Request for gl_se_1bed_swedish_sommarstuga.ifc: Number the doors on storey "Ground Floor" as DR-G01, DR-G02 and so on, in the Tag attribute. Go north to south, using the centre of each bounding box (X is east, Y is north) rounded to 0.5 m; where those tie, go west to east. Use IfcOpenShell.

First a look at what the model holds.

```python
import ifcopenshell
import ifcopenshell.util.element
import ifcopenshell.util.placement

model = ifcopenshell.open("gl_se_1bed_swedish_sommarstuga.ifc")
print(model.schema)
storey = next(s for s in model.by_type("IfcBuildingStorey") if s.Name == "Ground Floor")
doors = [e for e in ifcopenshell.util.element.get_decomposition(storey) if e.is_a("IfcDoor")]
for e in sorted(doors, key=lambda e: e.id()):
    origin = ifcopenshell.util.placement.get_local_placement(e.ObjectPlacement)[:3, 3]
    print(e.id(), e.Tag, e.Name, origin.round(2) + 0.0, sep=" | ")
```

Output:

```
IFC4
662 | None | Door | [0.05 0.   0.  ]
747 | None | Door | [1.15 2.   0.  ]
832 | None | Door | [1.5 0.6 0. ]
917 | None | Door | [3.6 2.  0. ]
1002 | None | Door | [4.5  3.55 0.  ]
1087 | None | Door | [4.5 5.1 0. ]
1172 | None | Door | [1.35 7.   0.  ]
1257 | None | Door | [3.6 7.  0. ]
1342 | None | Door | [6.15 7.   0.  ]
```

```python
import ifcopenshell
import ifcopenshell.geom
import ifcopenshell.util.element
import ifcopenshell.util.shape

model = ifcopenshell.open("gl_se_1bed_swedish_sommarstuga.ifc")
settings = ifcopenshell.geom.settings()
settings.set("use-world-coords", True)


def centre(element):
    shape = ifcopenshell.geom.create_shape(settings, element)
    return ifcopenshell.util.shape.get_bbox_centroid(shape.geometry)


storey = next(s for s in model.by_type("IfcBuildingStorey") if s.Name == "Ground Floor")
doors = [e for e in ifcopenshell.util.element.get_decomposition(storey) if e.is_a("IfcDoor")]

# Insertion points can sit at a corner or the storey origin, so sort by the geometry (in metres).
centres = {e: centre(e) for e in doors}
doors.sort(key=lambda e: (-round(centres[e][1] / 0.5), centres[e][0]))

for i, e in enumerate(doors, start=1):
    number = f"DR-G{i:02d}"
    e.Tag = number
    print(e.id(), number)

model.write("gl_se_1bed_swedish_sommarstuga_edited.ifc")
```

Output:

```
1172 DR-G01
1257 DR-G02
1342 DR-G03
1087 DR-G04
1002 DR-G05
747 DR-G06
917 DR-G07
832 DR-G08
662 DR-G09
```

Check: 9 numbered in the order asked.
